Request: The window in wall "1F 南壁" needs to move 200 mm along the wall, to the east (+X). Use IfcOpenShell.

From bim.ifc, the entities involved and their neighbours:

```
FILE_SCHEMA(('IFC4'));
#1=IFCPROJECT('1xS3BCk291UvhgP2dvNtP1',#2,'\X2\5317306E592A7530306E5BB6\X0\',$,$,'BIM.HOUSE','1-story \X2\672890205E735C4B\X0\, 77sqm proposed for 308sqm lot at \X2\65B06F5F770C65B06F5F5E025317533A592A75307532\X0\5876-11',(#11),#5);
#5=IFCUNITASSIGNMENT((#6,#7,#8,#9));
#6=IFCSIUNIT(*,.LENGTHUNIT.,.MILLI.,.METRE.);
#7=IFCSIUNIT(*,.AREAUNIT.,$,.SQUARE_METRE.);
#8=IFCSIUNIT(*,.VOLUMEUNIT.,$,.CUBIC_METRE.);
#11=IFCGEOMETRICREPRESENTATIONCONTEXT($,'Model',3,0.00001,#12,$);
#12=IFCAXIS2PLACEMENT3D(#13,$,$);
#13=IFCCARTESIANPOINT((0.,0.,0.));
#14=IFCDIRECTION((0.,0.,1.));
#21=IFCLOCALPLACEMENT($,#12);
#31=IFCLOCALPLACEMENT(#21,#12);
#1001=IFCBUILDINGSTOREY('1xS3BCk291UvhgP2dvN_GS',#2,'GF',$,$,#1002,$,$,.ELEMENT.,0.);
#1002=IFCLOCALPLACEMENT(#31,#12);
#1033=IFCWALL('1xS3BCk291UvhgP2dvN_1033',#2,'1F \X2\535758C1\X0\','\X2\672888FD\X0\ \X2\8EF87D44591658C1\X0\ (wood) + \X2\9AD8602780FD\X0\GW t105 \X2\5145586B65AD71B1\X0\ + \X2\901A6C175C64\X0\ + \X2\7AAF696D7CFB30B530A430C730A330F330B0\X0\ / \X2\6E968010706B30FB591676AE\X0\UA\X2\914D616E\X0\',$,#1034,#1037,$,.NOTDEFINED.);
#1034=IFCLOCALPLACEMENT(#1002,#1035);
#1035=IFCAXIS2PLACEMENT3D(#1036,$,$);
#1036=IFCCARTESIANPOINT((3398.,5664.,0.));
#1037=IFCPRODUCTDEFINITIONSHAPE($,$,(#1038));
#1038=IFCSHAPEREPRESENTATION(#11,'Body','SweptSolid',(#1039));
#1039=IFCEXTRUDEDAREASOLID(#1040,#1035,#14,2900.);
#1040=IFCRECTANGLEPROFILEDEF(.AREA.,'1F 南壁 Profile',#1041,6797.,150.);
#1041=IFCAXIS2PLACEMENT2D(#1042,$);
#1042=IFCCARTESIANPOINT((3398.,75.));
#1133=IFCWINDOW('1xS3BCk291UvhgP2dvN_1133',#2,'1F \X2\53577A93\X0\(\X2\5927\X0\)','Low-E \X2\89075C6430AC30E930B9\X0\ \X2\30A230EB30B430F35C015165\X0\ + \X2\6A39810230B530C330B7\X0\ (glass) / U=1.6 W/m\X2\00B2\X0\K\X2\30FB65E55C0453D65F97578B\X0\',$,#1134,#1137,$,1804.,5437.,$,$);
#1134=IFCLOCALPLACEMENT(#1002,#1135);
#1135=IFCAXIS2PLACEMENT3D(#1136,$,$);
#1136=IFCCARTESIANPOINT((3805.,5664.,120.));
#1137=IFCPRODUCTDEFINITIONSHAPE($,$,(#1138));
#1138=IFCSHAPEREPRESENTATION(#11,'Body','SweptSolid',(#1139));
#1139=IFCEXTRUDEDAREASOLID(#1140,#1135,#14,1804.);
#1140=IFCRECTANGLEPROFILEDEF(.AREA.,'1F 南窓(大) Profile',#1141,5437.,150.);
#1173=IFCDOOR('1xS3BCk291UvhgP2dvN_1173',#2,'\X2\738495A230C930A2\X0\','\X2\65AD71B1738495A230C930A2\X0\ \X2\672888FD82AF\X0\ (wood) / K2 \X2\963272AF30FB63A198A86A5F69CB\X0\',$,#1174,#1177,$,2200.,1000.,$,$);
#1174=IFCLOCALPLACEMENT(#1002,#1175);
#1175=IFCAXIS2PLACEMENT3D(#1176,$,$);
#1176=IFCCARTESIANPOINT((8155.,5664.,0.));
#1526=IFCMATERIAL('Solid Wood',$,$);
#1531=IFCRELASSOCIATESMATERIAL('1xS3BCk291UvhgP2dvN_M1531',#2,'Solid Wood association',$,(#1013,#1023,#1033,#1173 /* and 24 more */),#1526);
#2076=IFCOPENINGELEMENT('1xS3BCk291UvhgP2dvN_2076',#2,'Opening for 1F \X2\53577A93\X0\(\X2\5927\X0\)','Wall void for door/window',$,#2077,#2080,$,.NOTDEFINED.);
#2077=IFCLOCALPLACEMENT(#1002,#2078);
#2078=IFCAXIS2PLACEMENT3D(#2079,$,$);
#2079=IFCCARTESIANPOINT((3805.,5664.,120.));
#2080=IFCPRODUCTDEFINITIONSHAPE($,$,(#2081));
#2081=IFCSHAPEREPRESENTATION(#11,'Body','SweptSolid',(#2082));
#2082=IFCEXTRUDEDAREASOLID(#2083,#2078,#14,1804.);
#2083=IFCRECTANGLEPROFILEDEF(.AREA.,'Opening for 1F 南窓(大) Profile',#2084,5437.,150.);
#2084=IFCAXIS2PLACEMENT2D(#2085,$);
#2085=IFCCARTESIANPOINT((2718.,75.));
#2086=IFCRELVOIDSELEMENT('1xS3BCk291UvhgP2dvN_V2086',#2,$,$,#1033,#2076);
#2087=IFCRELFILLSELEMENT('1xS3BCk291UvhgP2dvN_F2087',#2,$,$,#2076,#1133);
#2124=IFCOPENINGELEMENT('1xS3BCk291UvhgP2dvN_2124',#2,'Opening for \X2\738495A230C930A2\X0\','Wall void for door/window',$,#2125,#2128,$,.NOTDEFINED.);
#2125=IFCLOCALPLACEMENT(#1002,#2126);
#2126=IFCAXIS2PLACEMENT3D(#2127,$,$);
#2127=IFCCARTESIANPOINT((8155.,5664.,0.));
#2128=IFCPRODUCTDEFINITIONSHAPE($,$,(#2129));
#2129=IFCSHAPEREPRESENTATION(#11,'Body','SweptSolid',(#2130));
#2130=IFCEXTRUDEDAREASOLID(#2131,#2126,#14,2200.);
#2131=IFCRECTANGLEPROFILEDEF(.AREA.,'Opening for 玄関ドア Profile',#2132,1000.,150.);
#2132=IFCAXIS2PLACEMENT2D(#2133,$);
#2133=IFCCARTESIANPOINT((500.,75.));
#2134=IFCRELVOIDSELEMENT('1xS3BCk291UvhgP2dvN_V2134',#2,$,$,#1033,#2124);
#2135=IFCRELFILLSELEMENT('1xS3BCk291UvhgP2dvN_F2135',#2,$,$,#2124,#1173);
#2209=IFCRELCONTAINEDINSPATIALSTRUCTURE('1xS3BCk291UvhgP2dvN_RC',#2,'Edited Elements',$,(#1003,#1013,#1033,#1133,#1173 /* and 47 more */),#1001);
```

```python
import ifcopenshell
import ifcopenshell.api.geometry
import ifcopenshell.util.placement
import ifcopenshell.util.unit

model = ifcopenshell.open("bim.ifc")
unit_scale = ifcopenshell.util.unit.calculate_unit_scale(model)

window = model.by_guid("1xS3BCk291UvhgP2dvN_1133")
opening = window.FillsVoids[0].RelatingOpeningElement
wall = opening.VoidsElements[0].RelatingBuildingElement

wall_matrix = ifcopenshell.util.placement.get_local_placement(wall.ObjectPlacement)
shift = wall_matrix[:3, 0] * 0.2 / unit_scale
before = ifcopenshell.util.placement.get_local_placement(window.ObjectPlacement)[:3, 3].copy()

# The window is not placed relative to its opening, so move both.
for product in (opening, window):
    matrix = ifcopenshell.util.placement.get_local_placement(product.ObjectPlacement)
    matrix[:3, 3] += shift
    ifcopenshell.api.geometry.edit_object_placement(model, product=product, matrix=matrix, is_si=False)

after = ifcopenshell.util.placement.get_local_placement(window.ObjectPlacement)[:3, 3]
print("window moved by", (after - before).round(3) + 0.0)

model.write("bim_edited.ifc")
```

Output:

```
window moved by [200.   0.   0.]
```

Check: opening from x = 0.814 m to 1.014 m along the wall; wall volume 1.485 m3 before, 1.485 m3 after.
